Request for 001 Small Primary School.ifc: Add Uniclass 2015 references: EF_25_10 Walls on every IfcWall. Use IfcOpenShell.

First a look at what the model holds.

```python
import ifcopenshell

model = ifcopenshell.open("001 Small Primary School.ifc")
print(model.schema)
print("classifications:", [c.Name for c in model.by_type("IfcClassification")])
for ifc_class in ("IfcDoor", "IfcRoof", "IfcStair", "IfcWall", "IfcWindow"):
    print(ifc_class, len(model.by_type(ifc_class)))
```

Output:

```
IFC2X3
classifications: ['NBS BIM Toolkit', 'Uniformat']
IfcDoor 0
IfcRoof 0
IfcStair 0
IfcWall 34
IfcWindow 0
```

```python
import ifcopenshell
import ifcopenshell.api.classification

model = ifcopenshell.open("001 Small Primary School.ifc")

# IFC2X3 requires Source and Edition and has no link from the project to the system.
system = model.create_entity("IfcClassification", Source="NBS", Edition="2015", Name="Uniclass 2015")

codes = {
    "IfcWall": ("EF_25_10", "Walls"),
}
for ifc_class, (code, name) in codes.items():
    products = model.by_type(ifc_class)
    ifcopenshell.api.classification.add_reference(
        model, products=products, classification=system, identification=code, name=name
    )
    print(code, len(products))

model.write("001 Small Primary School-out.ifc")
```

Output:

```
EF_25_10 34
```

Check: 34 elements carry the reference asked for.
